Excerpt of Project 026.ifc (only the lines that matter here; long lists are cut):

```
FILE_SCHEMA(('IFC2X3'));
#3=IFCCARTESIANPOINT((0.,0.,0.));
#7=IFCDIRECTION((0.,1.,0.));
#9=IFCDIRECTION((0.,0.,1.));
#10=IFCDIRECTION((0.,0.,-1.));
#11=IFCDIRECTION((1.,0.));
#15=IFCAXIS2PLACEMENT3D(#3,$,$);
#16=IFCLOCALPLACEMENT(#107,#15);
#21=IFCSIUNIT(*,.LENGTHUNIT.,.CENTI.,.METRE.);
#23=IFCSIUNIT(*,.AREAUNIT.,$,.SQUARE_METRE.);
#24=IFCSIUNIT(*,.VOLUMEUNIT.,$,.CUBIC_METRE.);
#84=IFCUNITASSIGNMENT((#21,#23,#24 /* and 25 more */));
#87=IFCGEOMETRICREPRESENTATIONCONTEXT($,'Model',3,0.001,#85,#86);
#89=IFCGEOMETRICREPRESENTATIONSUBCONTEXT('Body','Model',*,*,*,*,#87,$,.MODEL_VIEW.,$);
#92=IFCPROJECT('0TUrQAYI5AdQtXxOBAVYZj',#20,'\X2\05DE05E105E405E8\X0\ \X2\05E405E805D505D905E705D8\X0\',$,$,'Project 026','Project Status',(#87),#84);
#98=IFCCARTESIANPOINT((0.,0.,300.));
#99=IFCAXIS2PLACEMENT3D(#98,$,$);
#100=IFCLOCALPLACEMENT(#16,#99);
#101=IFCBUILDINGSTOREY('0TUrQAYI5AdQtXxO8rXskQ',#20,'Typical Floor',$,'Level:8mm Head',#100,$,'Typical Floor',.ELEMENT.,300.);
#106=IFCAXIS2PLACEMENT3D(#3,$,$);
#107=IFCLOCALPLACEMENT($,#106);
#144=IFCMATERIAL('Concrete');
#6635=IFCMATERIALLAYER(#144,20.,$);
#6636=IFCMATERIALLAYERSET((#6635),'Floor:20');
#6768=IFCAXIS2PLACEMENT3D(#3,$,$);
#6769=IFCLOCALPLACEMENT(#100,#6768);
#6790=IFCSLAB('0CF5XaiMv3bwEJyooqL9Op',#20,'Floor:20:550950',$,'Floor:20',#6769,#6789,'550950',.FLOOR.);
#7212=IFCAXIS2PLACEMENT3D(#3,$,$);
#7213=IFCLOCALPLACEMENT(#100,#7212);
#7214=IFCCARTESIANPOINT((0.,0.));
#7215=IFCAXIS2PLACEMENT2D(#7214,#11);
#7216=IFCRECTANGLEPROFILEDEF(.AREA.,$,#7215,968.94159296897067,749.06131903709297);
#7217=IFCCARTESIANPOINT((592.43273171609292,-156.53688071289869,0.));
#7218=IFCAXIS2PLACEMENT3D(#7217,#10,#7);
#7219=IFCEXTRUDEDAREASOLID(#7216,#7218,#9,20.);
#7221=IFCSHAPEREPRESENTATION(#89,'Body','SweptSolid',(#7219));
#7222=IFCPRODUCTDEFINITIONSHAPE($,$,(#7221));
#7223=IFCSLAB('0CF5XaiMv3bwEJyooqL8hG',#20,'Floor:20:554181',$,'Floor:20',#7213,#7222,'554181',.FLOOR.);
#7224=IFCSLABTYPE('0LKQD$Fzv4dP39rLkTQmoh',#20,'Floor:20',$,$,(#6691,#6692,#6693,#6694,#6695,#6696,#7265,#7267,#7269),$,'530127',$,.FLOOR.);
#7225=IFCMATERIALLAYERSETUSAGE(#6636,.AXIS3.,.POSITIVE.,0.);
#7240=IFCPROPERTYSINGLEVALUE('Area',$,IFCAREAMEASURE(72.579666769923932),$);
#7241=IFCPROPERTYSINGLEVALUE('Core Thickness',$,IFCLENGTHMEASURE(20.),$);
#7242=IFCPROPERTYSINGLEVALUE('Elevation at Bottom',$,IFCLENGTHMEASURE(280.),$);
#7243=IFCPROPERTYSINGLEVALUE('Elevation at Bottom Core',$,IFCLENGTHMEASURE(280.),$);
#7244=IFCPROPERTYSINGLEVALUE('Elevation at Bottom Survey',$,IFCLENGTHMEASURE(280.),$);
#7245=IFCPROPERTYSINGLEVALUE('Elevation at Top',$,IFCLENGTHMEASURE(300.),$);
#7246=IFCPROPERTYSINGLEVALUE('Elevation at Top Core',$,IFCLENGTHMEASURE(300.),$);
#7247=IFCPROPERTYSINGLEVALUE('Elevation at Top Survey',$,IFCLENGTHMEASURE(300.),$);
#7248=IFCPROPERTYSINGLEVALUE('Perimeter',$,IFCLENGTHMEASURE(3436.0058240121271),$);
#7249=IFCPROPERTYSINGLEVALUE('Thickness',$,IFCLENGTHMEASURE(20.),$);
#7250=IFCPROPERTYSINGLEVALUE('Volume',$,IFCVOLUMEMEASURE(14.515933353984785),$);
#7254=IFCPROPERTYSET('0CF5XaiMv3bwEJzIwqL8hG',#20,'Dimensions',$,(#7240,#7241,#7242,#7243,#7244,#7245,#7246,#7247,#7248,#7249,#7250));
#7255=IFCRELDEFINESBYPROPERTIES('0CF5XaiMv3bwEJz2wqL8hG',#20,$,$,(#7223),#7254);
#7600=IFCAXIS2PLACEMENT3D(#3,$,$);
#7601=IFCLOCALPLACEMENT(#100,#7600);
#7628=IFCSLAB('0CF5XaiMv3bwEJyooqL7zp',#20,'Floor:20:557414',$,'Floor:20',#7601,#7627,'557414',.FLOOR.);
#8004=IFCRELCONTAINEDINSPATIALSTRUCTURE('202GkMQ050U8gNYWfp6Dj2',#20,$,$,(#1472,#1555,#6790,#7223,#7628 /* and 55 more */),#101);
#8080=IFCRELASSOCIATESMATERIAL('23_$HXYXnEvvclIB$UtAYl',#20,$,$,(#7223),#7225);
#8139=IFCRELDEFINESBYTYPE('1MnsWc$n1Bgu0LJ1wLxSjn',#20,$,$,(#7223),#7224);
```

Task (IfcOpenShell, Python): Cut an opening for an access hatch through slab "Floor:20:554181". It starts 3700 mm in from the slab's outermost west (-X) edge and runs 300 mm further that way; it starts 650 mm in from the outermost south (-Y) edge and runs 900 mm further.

```python
import numpy as np
import ifcopenshell
import ifcopenshell.api.feature
import ifcopenshell.api.geometry
import ifcopenshell.api.pset
import ifcopenshell.api.root
import ifcopenshell.geom
import ifcopenshell.util.element
import ifcopenshell.util.placement
import ifcopenshell.util.representation
import ifcopenshell.util.shape
import ifcopenshell.util.unit

model = ifcopenshell.open("Project 026.ifc")
unit_scale = ifcopenshell.util.unit.calculate_unit_scale(model)
area_scale = ifcopenshell.util.unit.calculate_unit_scale(model, "AREAUNIT")
volume_scale = ifcopenshell.util.unit.calculate_unit_scale(model, "VOLUMEUNIT")
settings = ifcopenshell.geom.settings()


def volume(element):
    """Net volume in cubic metres, openings subtracted."""
    shape = ifcopenshell.geom.create_shape(settings, element)
    return ifcopenshell.util.shape.get_volume(shape.geometry)


slab = model.by_guid("0CF5XaiMv3bwEJyooqL8hG")
before = volume(slab)

# Extent in the slab's own axes, in metres. The edges named are its -X and -Y sides.
slab_shape = ifcopenshell.geom.create_shape(settings, slab)
vertices = ifcopenshell.util.shape.get_vertices(slab_shape.geometry)
x_min, y_min, bottom = vertices.min(axis=0)
top = vertices[:, 2].max()

opening = ifcopenshell.api.root.create_entity(model, ifc_class="IfcOpeningElement", name="Access hatch opening")
context = ifcopenshell.util.representation.get_context(model, "Model", "Body", "MODEL_VIEW")
width, depth = 0.3, 0.9
outline = [(0.0, 0.0), (width, 0.0), (width, depth), (0.0, depth), (0.0, 0.0)]
# Overshoot both faces by 50 mm so the cut is clean.
shape = ifcopenshell.api.geometry.add_slab_representation(
    model, context=context, depth=top - bottom + 0.1, polyline=outline
)
ifcopenshell.api.geometry.assign_representation(model, product=opening, representation=shape)

matrix = ifcopenshell.util.placement.get_local_placement(slab.ObjectPlacement)
matrix[:, 3] = matrix @ np.append(np.array([x_min + 3.7, y_min + 0.65, bottom - 0.05]) / unit_scale, 1.0)
ifcopenshell.api.geometry.edit_object_placement(model, product=opening, matrix=matrix, is_si=False)
ifcopenshell.api.feature.add_feature(model, feature=opening, element=slab)

after = volume(slab)

# Update the slab's stored quantities.
pset = model.by_id(ifcopenshell.util.element.get_pset(slab, "Dimensions", should_inherit=False)["id"])
ifcopenshell.api.pset.edit_pset(model, pset=pset, properties={
    "Area": model.create_entity("IfcAreaMeasure", after / (top - bottom) / area_scale),
    "Volume": model.create_entity("IfcVolumeMeasure", after / volume_scale),
})

print(f"slab volume {before:.3f} -> {after:.3f} m3")

model.write("Project 026_updated.ifc")
```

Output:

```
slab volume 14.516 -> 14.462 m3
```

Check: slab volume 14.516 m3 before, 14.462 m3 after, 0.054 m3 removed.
